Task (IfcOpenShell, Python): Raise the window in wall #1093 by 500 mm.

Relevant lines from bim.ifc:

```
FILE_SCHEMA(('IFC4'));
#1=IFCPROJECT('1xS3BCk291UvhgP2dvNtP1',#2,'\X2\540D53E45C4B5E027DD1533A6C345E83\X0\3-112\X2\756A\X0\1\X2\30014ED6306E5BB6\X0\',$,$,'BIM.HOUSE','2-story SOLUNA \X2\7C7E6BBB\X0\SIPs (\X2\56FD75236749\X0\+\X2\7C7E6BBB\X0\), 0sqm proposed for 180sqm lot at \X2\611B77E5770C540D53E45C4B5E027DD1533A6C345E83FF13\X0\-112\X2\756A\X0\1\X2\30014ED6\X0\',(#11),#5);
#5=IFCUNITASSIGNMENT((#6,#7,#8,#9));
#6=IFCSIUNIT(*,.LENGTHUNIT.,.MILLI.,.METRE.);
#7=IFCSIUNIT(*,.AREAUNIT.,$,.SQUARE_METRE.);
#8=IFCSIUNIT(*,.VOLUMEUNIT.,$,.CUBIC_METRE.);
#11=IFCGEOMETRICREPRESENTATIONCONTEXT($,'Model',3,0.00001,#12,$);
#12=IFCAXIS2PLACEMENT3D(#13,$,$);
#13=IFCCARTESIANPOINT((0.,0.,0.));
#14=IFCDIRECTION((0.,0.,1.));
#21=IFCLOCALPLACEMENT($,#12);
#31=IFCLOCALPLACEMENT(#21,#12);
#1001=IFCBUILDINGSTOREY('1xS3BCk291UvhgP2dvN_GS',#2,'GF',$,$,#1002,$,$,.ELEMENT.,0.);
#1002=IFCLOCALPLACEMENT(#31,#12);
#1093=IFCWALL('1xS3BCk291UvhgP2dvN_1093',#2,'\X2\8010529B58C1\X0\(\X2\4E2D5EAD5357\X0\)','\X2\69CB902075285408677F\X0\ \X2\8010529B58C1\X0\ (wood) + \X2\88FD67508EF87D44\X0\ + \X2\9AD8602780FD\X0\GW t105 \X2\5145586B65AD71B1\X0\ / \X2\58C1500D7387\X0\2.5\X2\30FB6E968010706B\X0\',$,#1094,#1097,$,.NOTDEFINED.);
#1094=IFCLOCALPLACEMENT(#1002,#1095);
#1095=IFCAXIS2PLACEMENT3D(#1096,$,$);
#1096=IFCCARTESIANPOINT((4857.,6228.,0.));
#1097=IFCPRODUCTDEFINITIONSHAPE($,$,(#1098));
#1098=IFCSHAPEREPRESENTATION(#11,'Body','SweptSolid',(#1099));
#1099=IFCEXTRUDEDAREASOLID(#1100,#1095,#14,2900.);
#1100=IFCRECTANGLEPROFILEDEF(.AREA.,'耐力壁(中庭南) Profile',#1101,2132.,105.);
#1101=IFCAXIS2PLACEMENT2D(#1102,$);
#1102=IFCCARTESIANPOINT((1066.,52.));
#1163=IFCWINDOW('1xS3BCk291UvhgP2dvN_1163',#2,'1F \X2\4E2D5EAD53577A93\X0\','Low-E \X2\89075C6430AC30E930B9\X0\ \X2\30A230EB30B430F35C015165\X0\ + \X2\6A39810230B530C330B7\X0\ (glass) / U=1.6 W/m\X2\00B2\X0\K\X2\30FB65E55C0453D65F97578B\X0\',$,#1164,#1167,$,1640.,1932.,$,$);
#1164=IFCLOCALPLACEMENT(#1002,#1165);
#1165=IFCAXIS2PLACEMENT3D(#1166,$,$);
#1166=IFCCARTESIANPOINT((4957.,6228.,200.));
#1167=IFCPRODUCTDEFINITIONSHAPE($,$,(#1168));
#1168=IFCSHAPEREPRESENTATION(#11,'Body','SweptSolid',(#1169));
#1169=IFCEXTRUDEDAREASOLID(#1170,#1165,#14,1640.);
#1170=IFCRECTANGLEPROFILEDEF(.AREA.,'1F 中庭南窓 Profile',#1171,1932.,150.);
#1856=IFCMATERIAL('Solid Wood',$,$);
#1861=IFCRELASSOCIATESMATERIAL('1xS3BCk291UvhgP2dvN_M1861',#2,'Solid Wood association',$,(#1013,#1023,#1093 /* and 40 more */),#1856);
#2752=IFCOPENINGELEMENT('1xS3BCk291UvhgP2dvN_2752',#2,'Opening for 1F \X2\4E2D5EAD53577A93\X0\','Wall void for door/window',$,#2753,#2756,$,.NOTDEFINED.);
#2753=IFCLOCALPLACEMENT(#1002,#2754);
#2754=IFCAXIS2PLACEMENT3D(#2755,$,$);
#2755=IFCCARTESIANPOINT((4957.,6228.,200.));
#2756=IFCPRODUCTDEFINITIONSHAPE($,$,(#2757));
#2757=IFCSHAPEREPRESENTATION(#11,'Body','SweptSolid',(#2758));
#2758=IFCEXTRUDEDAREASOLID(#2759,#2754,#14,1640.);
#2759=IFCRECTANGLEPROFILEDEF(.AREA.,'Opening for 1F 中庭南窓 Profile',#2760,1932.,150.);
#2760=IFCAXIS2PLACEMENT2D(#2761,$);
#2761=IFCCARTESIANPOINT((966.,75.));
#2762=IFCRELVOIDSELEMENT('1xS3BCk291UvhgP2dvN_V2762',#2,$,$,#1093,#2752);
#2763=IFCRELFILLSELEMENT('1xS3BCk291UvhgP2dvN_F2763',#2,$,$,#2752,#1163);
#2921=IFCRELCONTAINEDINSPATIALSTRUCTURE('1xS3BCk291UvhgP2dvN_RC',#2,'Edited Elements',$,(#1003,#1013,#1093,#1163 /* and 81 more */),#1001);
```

```python
import numpy as np
import ifcopenshell
import ifcopenshell.api.geometry
import ifcopenshell.util.placement
import ifcopenshell.util.unit

model = ifcopenshell.open("bim.ifc")
unit_scale = ifcopenshell.util.unit.calculate_unit_scale(model)

window = model.by_guid("1xS3BCk291UvhgP2dvN_1163")
opening = window.FillsVoids[0].RelatingOpeningElement
dz = 0.5 / unit_scale

shift = np.array([0.0, 0.0, dz])
# The window is not placed relative to its opening, so move both.
for product in (opening, window):
    matrix = ifcopenshell.util.placement.get_local_placement(product.ObjectPlacement)
    matrix[:3, 3] += shift
    ifcopenshell.api.geometry.edit_object_placement(model, product=product, matrix=matrix, is_si=False)

print(f"moved by {dz * unit_scale:+.3f} m")

model.write("bim_rev.ifc")
```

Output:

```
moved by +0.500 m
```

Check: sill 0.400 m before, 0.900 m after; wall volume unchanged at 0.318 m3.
